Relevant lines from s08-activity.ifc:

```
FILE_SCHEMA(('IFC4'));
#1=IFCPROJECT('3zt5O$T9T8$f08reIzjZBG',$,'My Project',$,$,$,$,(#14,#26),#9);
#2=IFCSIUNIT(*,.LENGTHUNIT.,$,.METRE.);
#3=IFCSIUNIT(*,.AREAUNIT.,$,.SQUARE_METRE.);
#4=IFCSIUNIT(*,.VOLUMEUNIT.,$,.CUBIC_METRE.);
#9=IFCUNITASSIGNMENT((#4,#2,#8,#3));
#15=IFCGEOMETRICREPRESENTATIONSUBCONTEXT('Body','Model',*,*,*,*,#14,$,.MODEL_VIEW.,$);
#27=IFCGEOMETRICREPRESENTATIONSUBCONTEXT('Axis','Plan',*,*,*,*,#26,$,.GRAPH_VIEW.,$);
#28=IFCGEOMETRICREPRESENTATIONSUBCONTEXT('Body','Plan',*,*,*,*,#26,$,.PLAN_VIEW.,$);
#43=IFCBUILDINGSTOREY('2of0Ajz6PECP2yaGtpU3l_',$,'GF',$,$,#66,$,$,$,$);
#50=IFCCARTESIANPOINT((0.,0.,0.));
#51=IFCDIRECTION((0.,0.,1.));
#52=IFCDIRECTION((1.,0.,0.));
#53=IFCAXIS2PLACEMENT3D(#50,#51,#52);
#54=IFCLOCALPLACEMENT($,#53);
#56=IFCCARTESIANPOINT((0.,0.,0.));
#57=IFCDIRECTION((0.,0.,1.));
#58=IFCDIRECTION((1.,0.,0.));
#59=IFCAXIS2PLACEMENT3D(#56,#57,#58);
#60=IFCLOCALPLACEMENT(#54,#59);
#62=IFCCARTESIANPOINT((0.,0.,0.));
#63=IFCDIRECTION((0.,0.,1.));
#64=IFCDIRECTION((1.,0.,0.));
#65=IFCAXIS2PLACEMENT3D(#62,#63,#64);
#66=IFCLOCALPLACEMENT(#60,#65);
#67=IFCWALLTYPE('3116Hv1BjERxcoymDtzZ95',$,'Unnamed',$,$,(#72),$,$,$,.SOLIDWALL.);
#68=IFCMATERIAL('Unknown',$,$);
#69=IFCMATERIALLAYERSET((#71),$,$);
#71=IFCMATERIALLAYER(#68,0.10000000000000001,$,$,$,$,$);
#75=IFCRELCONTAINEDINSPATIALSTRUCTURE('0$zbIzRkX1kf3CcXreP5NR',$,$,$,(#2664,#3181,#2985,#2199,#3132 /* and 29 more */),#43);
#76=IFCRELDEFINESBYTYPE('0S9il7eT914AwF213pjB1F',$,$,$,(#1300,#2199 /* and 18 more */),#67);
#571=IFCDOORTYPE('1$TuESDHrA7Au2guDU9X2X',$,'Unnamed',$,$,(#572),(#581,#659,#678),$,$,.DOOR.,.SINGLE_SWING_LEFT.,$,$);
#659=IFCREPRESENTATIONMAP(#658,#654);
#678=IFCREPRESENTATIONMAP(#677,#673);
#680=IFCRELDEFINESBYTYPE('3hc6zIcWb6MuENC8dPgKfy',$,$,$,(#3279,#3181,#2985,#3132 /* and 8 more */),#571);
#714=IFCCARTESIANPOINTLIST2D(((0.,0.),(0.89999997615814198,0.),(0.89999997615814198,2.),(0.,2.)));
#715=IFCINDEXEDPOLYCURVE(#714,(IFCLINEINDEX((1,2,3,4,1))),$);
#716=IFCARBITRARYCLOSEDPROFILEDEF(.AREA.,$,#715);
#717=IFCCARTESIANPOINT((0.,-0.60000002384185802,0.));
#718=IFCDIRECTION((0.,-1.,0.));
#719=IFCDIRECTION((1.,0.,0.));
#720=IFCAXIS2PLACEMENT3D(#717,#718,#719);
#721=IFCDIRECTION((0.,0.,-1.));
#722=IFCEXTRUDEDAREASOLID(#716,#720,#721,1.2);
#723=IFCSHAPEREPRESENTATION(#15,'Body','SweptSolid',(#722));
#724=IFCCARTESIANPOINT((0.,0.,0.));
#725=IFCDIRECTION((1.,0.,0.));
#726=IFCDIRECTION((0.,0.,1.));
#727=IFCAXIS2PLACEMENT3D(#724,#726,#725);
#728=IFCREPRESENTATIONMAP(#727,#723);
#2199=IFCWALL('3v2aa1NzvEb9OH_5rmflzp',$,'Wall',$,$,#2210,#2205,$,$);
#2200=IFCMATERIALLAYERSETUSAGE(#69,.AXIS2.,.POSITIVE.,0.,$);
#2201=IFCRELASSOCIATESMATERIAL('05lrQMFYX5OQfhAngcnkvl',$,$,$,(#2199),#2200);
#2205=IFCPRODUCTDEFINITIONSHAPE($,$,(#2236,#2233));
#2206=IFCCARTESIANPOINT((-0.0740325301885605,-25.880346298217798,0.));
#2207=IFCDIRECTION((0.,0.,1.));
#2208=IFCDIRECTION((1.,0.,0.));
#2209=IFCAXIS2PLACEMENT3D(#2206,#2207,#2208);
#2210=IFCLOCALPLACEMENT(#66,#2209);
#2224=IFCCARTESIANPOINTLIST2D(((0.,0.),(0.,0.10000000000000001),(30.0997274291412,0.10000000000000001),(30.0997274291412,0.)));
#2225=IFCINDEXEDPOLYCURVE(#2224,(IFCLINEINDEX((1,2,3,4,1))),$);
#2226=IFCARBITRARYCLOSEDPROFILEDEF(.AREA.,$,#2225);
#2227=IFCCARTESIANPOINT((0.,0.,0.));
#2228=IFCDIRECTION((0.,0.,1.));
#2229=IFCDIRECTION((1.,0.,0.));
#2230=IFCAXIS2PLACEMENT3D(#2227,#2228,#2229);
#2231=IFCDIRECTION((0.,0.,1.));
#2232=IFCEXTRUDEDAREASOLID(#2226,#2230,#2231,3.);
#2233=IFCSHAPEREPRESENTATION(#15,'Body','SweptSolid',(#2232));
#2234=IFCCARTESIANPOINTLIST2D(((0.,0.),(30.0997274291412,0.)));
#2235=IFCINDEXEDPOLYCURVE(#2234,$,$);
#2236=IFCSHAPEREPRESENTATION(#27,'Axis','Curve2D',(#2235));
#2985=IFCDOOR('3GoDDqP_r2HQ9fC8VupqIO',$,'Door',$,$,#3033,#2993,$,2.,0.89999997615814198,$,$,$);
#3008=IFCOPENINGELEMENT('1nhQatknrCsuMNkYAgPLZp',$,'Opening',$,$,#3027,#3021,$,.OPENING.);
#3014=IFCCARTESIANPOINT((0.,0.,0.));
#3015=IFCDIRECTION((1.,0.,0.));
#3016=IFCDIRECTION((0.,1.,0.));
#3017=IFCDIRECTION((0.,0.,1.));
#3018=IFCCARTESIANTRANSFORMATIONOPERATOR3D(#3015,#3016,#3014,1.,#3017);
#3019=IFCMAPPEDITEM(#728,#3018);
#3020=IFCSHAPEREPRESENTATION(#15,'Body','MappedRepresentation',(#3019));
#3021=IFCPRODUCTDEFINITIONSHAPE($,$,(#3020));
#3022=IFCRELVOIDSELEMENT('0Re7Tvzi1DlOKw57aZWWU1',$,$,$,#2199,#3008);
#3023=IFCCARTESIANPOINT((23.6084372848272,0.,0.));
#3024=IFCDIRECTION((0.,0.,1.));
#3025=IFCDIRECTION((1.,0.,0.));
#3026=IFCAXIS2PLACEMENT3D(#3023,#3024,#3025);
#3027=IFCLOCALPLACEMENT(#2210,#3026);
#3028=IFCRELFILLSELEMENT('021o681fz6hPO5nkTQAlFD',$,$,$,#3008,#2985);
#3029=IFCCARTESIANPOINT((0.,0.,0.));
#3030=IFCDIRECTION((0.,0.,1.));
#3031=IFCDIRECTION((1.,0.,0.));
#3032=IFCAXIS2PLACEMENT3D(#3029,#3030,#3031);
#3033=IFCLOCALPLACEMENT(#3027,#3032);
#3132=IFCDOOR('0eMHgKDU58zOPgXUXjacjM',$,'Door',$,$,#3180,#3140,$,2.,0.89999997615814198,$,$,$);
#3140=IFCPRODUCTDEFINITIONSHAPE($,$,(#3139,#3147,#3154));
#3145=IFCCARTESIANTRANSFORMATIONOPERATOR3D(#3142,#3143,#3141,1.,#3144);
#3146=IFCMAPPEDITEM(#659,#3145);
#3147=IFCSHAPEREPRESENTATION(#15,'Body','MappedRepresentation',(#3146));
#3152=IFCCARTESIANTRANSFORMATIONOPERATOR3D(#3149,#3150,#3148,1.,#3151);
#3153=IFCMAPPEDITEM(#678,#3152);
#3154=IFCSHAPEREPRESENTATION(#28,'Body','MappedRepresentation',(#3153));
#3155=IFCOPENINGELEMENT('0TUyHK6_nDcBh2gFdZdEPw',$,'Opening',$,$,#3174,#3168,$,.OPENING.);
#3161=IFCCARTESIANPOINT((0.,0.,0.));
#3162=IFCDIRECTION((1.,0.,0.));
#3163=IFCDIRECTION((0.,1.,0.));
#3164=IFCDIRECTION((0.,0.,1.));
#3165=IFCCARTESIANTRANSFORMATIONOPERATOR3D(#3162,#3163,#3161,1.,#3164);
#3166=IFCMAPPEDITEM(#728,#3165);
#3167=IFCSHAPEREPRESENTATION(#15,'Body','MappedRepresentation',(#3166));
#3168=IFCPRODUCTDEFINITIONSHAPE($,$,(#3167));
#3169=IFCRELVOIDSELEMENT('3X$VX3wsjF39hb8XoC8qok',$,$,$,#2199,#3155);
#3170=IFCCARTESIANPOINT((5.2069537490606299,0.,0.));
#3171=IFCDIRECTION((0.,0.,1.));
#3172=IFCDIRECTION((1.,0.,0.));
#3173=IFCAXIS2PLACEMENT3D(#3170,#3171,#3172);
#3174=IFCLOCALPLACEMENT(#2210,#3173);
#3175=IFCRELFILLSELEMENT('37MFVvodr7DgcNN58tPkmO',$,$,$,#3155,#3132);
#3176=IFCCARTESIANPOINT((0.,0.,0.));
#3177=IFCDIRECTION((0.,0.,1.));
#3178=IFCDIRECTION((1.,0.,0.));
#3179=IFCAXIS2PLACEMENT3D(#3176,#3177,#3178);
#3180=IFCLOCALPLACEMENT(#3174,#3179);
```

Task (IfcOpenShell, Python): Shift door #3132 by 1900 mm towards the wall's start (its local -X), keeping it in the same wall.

```python
import ifcopenshell
import ifcopenshell.api.geometry
import ifcopenshell.util.placement
import ifcopenshell.util.unit

model = ifcopenshell.open("s08-activity.ifc")
unit_scale = ifcopenshell.util.unit.calculate_unit_scale(model)

door = model.by_guid("0eMHgKDU58zOPgXUXjacjM")
opening = door.FillsVoids[0].RelatingOpeningElement
wall = opening.VoidsElements[0].RelatingBuildingElement

wall_matrix = ifcopenshell.util.placement.get_local_placement(wall.ObjectPlacement)
shift = wall_matrix[:3, 0] * -1.9 / unit_scale
before = ifcopenshell.util.placement.get_local_placement(door.ObjectPlacement)[:3, 3].copy()

# The door is placed relative to its opening, so it follows when the opening moves.
matrix = ifcopenshell.util.placement.get_local_placement(opening.ObjectPlacement)
matrix[:3, 3] += shift
ifcopenshell.api.geometry.edit_object_placement(
    model, product=opening, matrix=matrix, is_si=False, should_transform_children=True
)

after = ifcopenshell.util.placement.get_local_placement(door.ObjectPlacement)[:3, 3]
print("door moved by", (after - before).round(3) + 0.0)

model.write("s08-activity_edited.ifc")
```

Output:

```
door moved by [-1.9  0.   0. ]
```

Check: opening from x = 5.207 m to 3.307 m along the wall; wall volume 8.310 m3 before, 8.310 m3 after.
